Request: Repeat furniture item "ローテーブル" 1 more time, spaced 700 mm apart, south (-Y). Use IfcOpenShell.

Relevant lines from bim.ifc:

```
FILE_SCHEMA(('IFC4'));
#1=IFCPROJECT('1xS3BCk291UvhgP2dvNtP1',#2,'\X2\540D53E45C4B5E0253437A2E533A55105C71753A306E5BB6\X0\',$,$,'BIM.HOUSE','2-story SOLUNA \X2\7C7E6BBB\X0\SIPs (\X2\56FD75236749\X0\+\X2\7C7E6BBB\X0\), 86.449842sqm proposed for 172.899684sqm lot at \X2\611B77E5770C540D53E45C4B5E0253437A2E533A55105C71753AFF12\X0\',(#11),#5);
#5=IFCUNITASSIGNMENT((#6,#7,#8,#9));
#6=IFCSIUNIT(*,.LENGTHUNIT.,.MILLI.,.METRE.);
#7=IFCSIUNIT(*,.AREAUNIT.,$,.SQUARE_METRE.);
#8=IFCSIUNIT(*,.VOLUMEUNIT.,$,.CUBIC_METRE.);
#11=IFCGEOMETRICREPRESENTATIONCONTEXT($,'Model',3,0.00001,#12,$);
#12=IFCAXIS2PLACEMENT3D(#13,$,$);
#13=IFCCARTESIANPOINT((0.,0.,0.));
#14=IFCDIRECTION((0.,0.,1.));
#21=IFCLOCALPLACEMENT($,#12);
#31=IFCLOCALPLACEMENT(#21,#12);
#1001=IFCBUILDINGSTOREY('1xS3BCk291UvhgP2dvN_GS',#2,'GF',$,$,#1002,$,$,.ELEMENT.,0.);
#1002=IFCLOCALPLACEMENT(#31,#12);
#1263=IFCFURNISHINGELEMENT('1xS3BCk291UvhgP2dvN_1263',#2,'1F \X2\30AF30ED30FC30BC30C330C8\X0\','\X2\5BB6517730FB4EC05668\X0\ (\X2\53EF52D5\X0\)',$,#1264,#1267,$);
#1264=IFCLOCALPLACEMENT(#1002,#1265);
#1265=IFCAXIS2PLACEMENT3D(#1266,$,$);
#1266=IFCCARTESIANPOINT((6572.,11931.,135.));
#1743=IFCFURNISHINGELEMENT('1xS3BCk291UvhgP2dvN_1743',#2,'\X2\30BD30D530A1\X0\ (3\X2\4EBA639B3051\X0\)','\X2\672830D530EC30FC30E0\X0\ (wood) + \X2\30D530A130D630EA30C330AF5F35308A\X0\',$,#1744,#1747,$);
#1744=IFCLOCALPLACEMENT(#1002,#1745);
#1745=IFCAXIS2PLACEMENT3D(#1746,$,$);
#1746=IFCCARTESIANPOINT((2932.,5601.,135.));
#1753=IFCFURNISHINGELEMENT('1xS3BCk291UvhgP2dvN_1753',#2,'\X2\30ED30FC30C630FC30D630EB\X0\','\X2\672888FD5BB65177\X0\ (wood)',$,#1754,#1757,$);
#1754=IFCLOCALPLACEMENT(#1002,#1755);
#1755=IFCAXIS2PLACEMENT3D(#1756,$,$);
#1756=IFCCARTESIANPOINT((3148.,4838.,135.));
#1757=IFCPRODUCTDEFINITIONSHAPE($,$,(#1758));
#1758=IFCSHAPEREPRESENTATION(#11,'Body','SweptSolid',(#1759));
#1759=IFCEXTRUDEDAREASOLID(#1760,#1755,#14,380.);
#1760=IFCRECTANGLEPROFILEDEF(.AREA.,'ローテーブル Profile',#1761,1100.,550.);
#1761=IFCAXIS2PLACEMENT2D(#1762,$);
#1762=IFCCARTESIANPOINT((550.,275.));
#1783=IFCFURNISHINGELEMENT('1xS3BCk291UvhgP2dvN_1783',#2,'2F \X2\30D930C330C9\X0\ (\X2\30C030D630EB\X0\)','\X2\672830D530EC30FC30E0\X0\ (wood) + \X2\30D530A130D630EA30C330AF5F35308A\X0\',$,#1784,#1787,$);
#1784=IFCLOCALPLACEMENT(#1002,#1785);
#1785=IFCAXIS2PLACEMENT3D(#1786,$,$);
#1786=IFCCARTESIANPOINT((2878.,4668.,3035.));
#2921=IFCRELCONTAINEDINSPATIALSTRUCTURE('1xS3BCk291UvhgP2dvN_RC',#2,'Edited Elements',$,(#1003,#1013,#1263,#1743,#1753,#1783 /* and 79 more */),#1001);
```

```python
import numpy as np
import ifcopenshell
import ifcopenshell.api.geometry
import ifcopenshell.api.root
import ifcopenshell.util.element
import ifcopenshell.util.placement
import ifcopenshell.util.unit

model = ifcopenshell.open("bim.ifc")
unit_scale = ifcopenshell.util.unit.calculate_unit_scale(model)


def reuse_history(source, copy):
    """copy_class also copies each property set's owner history, people and application; keep the originals."""
    for rel in copy.IsDefinedBy:
        if rel.is_a("IfcRelDefinesByProperties") and (history := rel.RelatingPropertyDefinition.OwnerHistory):
            rel.RelatingPropertyDefinition.OwnerHistory = source.OwnerHistory
            ifcopenshell.util.element.remove_deep2(model, history)


source = model.by_id(1753)
base = ifcopenshell.util.placement.get_local_placement(source.ObjectPlacement)
step = np.array([0.0, -1.0, 0.0]) * 0.7 / unit_scale

for i in range(1, 2):
    copy = ifcopenshell.api.root.copy_class(model, product=source)
    copy.Representation = ifcopenshell.util.element.copy_deep(
        model, source.Representation, exclude=["IfcGeometricRepresentationContext", "IfcRepresentationMap"]
    )
    reuse_history(source, copy)
    matrix = base.copy()
    matrix[:3, 3] += i * step
    print("added at", matrix[:3, 3].round(3) + 0.0)
    ifcopenshell.api.geometry.edit_object_placement(model, product=copy, matrix=matrix, is_si=False)

model.write("bim_edited.ifc")
```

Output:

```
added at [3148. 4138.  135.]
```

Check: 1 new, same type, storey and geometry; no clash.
